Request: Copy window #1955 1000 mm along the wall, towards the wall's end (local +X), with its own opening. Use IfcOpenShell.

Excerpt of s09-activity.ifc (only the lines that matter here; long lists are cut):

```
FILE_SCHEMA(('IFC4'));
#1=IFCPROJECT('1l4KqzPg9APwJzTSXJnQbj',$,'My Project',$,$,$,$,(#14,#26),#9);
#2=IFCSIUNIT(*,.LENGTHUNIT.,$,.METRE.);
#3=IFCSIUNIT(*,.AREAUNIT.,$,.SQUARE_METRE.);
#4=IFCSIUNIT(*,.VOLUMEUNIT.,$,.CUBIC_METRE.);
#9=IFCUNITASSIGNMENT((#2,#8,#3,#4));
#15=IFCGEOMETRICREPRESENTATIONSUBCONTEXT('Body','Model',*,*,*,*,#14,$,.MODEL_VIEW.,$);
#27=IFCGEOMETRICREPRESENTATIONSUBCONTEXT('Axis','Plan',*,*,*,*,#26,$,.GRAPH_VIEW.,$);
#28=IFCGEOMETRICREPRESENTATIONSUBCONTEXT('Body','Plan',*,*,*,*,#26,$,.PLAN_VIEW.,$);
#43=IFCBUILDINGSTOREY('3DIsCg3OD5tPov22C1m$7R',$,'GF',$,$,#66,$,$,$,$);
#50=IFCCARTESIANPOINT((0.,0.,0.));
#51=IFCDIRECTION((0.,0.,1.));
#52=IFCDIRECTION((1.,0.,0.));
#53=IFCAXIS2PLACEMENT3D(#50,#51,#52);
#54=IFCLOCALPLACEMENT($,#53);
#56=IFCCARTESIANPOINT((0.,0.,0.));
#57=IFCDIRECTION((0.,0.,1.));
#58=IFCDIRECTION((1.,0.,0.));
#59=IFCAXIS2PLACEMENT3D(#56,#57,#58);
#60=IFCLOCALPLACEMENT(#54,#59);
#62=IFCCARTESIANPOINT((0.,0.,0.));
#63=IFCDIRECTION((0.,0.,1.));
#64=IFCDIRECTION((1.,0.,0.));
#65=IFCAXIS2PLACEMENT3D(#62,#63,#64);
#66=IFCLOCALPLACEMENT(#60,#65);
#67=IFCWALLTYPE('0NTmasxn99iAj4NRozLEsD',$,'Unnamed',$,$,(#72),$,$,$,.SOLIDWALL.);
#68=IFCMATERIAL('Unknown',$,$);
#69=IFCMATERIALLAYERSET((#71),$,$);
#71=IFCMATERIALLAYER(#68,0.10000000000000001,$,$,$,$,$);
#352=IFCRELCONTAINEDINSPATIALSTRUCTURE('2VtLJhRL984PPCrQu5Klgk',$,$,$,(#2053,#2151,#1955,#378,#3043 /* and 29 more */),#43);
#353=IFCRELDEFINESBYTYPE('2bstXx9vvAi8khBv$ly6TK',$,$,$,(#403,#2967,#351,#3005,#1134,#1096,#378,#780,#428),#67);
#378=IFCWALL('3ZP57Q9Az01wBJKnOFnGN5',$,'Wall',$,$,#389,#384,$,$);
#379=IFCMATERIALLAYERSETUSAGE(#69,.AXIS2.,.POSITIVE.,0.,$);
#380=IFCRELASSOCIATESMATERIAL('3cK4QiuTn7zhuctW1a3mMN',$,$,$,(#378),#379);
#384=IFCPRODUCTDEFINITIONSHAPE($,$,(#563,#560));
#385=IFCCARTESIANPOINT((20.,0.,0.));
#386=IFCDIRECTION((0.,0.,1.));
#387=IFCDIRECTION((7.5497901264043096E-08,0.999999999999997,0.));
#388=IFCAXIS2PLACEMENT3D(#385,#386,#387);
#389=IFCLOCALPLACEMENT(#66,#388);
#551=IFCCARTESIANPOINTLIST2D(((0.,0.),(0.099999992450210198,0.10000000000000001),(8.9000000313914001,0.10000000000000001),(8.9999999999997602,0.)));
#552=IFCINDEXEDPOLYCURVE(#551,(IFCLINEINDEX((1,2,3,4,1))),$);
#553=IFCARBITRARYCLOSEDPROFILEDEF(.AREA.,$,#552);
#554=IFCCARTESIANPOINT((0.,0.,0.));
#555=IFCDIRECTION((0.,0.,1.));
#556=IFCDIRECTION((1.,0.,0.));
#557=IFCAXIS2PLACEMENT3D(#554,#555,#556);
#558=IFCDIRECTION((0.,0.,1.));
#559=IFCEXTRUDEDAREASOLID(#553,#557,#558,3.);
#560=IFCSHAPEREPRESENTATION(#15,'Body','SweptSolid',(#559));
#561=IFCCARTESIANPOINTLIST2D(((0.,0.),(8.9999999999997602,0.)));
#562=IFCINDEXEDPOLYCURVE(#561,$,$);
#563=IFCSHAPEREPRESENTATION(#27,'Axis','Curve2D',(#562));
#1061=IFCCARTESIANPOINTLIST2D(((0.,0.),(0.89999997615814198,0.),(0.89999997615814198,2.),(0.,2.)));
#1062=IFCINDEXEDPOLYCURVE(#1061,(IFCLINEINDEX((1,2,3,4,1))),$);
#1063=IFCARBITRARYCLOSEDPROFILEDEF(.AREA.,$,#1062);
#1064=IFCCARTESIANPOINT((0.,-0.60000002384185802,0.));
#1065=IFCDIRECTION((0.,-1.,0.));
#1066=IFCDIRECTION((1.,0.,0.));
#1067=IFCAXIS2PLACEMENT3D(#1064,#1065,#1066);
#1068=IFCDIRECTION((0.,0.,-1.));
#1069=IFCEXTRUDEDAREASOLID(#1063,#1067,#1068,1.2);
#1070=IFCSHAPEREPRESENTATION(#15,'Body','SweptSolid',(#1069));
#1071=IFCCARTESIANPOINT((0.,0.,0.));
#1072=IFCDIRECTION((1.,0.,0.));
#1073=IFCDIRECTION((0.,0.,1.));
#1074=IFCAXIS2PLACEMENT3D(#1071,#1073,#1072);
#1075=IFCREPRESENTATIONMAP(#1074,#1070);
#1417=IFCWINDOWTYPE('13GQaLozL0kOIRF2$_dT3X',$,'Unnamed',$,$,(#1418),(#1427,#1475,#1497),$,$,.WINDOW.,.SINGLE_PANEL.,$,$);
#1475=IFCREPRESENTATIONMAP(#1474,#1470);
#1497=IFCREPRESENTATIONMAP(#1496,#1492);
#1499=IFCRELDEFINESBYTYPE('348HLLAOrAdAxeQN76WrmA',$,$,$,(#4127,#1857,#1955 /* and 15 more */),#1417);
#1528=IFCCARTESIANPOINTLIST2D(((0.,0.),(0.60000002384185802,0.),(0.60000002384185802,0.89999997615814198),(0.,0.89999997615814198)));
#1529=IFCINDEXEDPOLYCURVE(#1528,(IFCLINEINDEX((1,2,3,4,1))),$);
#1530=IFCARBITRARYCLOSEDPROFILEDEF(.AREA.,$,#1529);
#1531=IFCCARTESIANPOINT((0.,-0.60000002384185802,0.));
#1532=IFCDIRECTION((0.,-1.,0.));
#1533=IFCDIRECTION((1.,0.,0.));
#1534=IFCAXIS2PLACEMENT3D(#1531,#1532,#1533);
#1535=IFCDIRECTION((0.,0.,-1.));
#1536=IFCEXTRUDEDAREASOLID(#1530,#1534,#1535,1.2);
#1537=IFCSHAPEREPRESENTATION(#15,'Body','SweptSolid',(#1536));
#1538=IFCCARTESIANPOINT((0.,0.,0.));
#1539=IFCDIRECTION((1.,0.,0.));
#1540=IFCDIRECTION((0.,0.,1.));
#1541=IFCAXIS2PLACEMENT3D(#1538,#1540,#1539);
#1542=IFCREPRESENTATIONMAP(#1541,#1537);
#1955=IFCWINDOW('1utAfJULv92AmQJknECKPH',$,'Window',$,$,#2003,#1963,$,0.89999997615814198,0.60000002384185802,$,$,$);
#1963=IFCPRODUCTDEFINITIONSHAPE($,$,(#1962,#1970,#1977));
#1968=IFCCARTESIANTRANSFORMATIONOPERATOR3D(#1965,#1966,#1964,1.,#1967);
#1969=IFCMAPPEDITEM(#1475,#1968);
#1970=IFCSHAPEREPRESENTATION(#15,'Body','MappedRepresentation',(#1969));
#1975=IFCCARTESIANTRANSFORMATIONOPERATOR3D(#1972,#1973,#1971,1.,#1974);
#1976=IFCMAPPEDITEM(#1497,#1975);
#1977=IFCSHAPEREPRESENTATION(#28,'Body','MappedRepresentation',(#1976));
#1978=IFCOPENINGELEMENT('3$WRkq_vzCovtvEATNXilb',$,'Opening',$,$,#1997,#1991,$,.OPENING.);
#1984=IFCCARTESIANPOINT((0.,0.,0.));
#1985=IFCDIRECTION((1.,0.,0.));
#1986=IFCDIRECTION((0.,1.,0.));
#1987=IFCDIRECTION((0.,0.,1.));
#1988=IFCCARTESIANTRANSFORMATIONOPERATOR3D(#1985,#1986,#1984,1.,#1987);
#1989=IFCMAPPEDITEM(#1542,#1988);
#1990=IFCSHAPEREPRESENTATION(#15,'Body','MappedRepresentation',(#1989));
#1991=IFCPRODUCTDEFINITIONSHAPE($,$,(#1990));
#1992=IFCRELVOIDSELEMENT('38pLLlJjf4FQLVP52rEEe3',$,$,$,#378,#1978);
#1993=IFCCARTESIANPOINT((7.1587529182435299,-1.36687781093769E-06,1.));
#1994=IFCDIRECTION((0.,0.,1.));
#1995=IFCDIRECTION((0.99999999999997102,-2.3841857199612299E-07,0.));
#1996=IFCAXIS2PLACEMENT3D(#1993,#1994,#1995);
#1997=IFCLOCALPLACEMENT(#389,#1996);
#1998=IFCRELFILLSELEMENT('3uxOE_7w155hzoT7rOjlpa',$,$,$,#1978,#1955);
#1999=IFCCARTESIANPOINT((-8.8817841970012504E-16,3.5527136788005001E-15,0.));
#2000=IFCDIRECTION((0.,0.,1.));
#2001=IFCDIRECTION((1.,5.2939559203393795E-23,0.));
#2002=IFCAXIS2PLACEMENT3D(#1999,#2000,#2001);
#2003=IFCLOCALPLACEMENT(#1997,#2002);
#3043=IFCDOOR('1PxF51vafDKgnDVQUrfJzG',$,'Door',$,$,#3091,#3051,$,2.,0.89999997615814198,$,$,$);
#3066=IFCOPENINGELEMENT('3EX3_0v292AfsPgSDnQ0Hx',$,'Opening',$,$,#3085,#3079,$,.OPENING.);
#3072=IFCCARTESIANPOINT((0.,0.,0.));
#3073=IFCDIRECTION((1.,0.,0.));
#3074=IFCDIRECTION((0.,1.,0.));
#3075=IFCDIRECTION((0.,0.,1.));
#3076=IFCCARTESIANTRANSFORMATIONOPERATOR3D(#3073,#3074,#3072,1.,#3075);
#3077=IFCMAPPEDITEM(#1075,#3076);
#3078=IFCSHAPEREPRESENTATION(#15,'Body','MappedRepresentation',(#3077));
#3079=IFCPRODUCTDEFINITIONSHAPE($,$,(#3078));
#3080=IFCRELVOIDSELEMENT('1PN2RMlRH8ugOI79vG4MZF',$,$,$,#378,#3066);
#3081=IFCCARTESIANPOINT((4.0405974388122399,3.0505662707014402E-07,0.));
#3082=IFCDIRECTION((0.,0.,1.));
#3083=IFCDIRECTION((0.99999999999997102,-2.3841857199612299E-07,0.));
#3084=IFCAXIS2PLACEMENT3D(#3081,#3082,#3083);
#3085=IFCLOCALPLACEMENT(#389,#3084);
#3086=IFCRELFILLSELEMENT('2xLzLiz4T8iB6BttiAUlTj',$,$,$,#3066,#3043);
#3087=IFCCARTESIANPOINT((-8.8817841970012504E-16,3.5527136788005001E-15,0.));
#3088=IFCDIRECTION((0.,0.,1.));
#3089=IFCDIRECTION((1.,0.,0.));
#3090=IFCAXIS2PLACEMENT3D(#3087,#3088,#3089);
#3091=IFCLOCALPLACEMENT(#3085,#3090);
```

```python
import ifcopenshell
import ifcopenshell.api.feature
import ifcopenshell.api.geometry
import ifcopenshell.api.root
import ifcopenshell.geom
import ifcopenshell.util.element
import ifcopenshell.util.placement
import ifcopenshell.util.shape
import ifcopenshell.util.unit

model = ifcopenshell.open("s09-activity.ifc")
unit_scale = ifcopenshell.util.unit.calculate_unit_scale(model)
settings = ifcopenshell.geom.settings()


def volume(element):
    """Net volume in cubic metres, openings subtracted."""
    shape = ifcopenshell.geom.create_shape(settings, element)
    return ifcopenshell.util.shape.get_volume(shape.geometry)


window = model.by_id(1955)
opening = window.FillsVoids[0].RelatingOpeningElement
wall = opening.VoidsElements[0].RelatingBuildingElement
before = volume(wall)
shift = ifcopenshell.util.placement.get_local_placement(wall.ObjectPlacement)[:3, 0] * 1 / unit_scale

# copy_class copies the void relationship, type, container and properties, but no geometry.
new_opening = ifcopenshell.api.root.copy_class(model, product=opening)
new_opening.Representation = ifcopenshell.util.element.copy_deep(
    model, opening.Representation, exclude=["IfcGeometricRepresentationContext", "IfcRepresentationMap"]
)
new_window = ifcopenshell.api.root.copy_class(model, product=window)
new_window.Representation = ifcopenshell.util.element.copy_deep(
    model, window.Representation, exclude=["IfcGeometricRepresentationContext", "IfcRepresentationMap"]
)
ifcopenshell.api.feature.add_filling(model, opening=new_opening, element=new_window)

for old, new in ((opening, new_opening), (window, new_window)):
    matrix = ifcopenshell.util.placement.get_local_placement(old.ObjectPlacement)
    matrix[:3, 3] += shift
    ifcopenshell.api.geometry.edit_object_placement(model, product=new, matrix=matrix, is_si=False)

after = volume(wall)

print(f"wall volume {before:.3f} -> {after:.3f} m3")

model.write("s09-activity_v2.ifc")
```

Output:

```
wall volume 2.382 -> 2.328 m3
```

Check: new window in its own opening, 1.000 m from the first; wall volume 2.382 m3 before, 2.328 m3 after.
